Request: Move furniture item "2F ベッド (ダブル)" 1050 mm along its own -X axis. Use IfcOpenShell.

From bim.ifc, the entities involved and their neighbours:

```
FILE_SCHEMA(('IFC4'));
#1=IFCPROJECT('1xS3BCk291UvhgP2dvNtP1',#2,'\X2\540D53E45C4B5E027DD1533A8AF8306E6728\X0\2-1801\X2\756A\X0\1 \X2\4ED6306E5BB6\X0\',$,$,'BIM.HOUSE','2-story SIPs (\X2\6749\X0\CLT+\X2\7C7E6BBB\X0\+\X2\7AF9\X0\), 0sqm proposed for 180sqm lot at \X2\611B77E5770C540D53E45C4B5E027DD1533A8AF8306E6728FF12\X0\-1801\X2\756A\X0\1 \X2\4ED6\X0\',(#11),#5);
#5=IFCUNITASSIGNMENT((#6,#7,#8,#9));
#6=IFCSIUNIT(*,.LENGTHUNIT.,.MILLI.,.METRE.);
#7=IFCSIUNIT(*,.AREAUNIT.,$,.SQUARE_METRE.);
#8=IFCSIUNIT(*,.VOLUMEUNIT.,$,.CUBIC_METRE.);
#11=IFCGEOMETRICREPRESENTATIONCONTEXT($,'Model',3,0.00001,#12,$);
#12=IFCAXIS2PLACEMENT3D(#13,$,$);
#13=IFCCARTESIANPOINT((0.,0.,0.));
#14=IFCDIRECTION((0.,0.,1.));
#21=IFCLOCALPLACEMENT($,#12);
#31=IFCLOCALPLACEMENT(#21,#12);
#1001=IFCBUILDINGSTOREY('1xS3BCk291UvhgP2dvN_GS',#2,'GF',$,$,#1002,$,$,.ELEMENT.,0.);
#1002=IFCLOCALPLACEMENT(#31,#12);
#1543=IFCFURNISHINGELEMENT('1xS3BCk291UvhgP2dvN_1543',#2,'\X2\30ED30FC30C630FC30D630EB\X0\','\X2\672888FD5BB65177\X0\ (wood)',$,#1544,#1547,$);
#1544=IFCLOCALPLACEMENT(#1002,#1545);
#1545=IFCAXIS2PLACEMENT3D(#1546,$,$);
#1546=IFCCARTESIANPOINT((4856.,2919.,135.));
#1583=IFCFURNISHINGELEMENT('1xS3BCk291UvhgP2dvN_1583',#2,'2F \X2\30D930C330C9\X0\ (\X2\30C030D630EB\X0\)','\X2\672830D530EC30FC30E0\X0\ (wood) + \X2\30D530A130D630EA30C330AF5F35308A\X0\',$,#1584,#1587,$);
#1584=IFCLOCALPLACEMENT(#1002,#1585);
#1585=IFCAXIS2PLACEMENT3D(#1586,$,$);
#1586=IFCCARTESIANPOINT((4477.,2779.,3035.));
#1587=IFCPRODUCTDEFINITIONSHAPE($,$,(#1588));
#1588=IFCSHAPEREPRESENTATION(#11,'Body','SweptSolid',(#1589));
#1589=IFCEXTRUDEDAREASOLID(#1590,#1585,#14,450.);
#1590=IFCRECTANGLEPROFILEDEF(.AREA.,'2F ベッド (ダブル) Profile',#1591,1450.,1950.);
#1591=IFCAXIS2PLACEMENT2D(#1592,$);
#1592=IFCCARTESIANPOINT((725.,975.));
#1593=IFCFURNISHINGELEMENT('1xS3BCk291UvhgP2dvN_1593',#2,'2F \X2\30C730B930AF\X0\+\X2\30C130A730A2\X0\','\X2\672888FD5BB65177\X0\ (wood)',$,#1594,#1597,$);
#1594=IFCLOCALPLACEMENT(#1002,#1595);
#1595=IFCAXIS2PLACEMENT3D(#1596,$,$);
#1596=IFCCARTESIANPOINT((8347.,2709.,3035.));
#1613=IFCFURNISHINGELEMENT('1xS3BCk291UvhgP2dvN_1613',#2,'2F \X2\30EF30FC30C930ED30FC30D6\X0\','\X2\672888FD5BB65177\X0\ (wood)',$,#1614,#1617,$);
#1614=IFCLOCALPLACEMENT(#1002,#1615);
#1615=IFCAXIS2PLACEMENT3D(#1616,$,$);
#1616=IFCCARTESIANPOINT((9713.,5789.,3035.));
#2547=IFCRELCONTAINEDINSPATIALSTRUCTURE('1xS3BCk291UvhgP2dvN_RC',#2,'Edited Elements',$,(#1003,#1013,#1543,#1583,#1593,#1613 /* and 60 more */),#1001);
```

```python
import ifcopenshell
import ifcopenshell.api.geometry
import ifcopenshell.util.placement
import ifcopenshell.util.unit

model = ifcopenshell.open("bim.ifc")
unit_scale = ifcopenshell.util.unit.calculate_unit_scale(model)

item = model.by_guid("1xS3BCk291UvhgP2dvN_1583")
matrix = ifcopenshell.util.placement.get_local_placement(item.ObjectPlacement)
matrix[:3, 3] -= matrix[:3, 0] * 1.05 / unit_scale
ifcopenshell.api.geometry.edit_object_placement(model, product=item, matrix=matrix, is_si=False)

print(ifcopenshell.util.placement.get_local_placement(item.ObjectPlacement).round(3) + 0.0)

model.write("bim_rev.ifc")
```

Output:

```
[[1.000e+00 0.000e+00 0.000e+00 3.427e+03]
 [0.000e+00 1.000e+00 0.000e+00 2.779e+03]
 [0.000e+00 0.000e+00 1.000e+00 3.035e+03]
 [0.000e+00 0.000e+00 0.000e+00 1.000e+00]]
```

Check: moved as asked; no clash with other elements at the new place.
